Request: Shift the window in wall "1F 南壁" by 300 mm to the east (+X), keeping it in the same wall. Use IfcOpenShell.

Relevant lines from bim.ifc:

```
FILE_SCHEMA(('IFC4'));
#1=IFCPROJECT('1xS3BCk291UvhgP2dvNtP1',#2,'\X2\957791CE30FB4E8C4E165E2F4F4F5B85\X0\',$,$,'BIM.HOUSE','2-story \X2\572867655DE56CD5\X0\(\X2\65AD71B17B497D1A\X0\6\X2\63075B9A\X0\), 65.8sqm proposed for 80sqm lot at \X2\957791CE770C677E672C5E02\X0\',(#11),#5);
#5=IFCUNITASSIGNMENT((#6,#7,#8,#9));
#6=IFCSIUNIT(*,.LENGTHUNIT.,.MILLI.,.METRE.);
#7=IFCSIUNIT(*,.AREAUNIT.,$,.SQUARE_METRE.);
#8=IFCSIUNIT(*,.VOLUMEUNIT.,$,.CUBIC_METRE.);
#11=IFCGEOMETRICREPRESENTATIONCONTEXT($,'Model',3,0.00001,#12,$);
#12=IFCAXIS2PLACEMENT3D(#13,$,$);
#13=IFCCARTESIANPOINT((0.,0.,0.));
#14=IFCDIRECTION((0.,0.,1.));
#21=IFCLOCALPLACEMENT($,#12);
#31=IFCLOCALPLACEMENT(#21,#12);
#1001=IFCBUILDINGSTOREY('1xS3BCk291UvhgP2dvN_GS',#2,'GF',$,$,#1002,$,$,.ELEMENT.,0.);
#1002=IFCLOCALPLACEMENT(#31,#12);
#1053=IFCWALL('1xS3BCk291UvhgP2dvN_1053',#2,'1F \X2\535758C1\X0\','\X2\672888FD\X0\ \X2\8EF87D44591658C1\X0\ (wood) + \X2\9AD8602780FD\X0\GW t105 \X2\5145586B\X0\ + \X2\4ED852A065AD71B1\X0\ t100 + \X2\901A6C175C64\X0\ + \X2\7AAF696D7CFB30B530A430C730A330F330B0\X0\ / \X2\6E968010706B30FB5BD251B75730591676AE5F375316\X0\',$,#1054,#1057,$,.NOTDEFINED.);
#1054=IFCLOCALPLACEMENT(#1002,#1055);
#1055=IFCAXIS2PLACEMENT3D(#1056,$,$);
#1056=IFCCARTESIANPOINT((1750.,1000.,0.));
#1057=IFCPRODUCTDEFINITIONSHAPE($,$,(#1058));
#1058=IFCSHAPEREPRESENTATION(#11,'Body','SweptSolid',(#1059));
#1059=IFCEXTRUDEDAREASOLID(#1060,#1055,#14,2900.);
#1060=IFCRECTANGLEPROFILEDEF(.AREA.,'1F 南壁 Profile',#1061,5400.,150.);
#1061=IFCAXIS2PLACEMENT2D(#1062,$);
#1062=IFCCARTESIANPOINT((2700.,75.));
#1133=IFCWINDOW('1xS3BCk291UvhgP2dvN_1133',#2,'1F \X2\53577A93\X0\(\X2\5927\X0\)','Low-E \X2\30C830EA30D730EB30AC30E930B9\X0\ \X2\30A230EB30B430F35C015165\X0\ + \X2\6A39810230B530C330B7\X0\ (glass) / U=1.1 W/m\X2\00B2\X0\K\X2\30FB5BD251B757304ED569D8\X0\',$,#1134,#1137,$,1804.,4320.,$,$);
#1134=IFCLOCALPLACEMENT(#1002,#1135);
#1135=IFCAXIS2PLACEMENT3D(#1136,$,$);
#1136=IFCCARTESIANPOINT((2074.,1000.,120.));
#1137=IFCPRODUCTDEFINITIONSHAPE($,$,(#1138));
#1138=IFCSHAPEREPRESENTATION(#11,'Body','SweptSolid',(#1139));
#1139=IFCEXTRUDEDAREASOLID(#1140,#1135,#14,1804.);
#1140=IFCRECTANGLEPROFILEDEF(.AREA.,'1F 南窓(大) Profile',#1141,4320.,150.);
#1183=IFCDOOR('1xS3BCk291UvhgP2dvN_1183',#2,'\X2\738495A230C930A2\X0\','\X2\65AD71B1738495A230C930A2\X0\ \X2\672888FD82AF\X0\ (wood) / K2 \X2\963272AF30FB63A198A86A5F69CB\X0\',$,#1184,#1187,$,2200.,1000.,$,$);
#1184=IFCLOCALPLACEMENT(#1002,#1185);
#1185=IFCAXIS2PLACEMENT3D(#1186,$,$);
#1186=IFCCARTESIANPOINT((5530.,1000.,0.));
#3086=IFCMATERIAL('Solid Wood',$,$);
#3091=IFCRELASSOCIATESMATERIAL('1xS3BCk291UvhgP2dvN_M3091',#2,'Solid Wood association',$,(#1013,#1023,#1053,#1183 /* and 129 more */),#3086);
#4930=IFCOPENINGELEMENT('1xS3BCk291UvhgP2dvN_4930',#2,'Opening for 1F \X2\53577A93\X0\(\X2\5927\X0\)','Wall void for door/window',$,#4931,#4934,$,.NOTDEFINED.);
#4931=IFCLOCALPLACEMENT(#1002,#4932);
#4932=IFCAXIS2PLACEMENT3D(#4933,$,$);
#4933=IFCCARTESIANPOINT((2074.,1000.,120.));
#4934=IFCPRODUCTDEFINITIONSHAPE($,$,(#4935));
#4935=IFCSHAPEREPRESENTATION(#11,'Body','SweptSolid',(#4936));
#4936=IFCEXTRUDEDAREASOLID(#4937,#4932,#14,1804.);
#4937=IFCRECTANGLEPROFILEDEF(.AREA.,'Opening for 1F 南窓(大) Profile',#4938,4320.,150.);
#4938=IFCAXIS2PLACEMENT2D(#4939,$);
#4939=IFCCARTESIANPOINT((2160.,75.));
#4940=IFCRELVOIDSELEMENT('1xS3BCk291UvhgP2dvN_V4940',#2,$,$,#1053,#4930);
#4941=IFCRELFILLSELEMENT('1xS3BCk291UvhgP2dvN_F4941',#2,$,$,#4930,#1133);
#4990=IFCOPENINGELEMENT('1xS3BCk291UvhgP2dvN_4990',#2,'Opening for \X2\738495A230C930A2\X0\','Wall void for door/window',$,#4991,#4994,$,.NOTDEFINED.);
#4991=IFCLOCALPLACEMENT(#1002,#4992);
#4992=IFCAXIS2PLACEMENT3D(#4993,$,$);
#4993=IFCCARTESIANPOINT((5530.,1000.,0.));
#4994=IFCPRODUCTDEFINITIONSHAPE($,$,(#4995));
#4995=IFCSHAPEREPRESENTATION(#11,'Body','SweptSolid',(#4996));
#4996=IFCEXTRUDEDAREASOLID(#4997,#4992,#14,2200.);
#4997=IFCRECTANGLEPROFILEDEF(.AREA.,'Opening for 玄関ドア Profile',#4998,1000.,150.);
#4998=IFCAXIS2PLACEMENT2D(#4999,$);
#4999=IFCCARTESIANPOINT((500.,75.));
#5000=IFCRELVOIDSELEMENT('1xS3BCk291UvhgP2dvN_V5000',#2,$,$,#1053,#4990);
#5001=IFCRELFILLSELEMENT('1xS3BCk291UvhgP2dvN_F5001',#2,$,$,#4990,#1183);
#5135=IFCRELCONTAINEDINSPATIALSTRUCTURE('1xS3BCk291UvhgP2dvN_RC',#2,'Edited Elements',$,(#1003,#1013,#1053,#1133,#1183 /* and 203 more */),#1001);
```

```python
import ifcopenshell
import ifcopenshell.api.geometry
import ifcopenshell.util.placement

model = ifcopenshell.open("bim.ifc")

window = model.by_guid("1xS3BCk291UvhgP2dvN_1133")
opening = window.FillsVoids[0].RelatingOpeningElement
wall = opening.VoidsElements[0].RelatingBuildingElement

wall_matrix = ifcopenshell.util.placement.get_local_placement(wall.ObjectPlacement)
shift = wall_matrix[:3, 0] * 300.0
before = ifcopenshell.util.placement.get_local_placement(window.ObjectPlacement)[:3, 3].copy()

# The window is not placed relative to its opening, so move both.
for product in (opening, window):
    matrix = ifcopenshell.util.placement.get_local_placement(product.ObjectPlacement)
    matrix[:3, 3] += shift
    ifcopenshell.api.geometry.edit_object_placement(model, product=product, matrix=matrix, is_si=False)

after = ifcopenshell.util.placement.get_local_placement(window.ObjectPlacement)[:3, 3]
print("window moved by", (after - before).round(3) + 0.0)

model.write("bim_v2.ifc")
```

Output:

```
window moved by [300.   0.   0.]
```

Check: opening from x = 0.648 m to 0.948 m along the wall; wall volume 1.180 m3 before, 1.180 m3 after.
